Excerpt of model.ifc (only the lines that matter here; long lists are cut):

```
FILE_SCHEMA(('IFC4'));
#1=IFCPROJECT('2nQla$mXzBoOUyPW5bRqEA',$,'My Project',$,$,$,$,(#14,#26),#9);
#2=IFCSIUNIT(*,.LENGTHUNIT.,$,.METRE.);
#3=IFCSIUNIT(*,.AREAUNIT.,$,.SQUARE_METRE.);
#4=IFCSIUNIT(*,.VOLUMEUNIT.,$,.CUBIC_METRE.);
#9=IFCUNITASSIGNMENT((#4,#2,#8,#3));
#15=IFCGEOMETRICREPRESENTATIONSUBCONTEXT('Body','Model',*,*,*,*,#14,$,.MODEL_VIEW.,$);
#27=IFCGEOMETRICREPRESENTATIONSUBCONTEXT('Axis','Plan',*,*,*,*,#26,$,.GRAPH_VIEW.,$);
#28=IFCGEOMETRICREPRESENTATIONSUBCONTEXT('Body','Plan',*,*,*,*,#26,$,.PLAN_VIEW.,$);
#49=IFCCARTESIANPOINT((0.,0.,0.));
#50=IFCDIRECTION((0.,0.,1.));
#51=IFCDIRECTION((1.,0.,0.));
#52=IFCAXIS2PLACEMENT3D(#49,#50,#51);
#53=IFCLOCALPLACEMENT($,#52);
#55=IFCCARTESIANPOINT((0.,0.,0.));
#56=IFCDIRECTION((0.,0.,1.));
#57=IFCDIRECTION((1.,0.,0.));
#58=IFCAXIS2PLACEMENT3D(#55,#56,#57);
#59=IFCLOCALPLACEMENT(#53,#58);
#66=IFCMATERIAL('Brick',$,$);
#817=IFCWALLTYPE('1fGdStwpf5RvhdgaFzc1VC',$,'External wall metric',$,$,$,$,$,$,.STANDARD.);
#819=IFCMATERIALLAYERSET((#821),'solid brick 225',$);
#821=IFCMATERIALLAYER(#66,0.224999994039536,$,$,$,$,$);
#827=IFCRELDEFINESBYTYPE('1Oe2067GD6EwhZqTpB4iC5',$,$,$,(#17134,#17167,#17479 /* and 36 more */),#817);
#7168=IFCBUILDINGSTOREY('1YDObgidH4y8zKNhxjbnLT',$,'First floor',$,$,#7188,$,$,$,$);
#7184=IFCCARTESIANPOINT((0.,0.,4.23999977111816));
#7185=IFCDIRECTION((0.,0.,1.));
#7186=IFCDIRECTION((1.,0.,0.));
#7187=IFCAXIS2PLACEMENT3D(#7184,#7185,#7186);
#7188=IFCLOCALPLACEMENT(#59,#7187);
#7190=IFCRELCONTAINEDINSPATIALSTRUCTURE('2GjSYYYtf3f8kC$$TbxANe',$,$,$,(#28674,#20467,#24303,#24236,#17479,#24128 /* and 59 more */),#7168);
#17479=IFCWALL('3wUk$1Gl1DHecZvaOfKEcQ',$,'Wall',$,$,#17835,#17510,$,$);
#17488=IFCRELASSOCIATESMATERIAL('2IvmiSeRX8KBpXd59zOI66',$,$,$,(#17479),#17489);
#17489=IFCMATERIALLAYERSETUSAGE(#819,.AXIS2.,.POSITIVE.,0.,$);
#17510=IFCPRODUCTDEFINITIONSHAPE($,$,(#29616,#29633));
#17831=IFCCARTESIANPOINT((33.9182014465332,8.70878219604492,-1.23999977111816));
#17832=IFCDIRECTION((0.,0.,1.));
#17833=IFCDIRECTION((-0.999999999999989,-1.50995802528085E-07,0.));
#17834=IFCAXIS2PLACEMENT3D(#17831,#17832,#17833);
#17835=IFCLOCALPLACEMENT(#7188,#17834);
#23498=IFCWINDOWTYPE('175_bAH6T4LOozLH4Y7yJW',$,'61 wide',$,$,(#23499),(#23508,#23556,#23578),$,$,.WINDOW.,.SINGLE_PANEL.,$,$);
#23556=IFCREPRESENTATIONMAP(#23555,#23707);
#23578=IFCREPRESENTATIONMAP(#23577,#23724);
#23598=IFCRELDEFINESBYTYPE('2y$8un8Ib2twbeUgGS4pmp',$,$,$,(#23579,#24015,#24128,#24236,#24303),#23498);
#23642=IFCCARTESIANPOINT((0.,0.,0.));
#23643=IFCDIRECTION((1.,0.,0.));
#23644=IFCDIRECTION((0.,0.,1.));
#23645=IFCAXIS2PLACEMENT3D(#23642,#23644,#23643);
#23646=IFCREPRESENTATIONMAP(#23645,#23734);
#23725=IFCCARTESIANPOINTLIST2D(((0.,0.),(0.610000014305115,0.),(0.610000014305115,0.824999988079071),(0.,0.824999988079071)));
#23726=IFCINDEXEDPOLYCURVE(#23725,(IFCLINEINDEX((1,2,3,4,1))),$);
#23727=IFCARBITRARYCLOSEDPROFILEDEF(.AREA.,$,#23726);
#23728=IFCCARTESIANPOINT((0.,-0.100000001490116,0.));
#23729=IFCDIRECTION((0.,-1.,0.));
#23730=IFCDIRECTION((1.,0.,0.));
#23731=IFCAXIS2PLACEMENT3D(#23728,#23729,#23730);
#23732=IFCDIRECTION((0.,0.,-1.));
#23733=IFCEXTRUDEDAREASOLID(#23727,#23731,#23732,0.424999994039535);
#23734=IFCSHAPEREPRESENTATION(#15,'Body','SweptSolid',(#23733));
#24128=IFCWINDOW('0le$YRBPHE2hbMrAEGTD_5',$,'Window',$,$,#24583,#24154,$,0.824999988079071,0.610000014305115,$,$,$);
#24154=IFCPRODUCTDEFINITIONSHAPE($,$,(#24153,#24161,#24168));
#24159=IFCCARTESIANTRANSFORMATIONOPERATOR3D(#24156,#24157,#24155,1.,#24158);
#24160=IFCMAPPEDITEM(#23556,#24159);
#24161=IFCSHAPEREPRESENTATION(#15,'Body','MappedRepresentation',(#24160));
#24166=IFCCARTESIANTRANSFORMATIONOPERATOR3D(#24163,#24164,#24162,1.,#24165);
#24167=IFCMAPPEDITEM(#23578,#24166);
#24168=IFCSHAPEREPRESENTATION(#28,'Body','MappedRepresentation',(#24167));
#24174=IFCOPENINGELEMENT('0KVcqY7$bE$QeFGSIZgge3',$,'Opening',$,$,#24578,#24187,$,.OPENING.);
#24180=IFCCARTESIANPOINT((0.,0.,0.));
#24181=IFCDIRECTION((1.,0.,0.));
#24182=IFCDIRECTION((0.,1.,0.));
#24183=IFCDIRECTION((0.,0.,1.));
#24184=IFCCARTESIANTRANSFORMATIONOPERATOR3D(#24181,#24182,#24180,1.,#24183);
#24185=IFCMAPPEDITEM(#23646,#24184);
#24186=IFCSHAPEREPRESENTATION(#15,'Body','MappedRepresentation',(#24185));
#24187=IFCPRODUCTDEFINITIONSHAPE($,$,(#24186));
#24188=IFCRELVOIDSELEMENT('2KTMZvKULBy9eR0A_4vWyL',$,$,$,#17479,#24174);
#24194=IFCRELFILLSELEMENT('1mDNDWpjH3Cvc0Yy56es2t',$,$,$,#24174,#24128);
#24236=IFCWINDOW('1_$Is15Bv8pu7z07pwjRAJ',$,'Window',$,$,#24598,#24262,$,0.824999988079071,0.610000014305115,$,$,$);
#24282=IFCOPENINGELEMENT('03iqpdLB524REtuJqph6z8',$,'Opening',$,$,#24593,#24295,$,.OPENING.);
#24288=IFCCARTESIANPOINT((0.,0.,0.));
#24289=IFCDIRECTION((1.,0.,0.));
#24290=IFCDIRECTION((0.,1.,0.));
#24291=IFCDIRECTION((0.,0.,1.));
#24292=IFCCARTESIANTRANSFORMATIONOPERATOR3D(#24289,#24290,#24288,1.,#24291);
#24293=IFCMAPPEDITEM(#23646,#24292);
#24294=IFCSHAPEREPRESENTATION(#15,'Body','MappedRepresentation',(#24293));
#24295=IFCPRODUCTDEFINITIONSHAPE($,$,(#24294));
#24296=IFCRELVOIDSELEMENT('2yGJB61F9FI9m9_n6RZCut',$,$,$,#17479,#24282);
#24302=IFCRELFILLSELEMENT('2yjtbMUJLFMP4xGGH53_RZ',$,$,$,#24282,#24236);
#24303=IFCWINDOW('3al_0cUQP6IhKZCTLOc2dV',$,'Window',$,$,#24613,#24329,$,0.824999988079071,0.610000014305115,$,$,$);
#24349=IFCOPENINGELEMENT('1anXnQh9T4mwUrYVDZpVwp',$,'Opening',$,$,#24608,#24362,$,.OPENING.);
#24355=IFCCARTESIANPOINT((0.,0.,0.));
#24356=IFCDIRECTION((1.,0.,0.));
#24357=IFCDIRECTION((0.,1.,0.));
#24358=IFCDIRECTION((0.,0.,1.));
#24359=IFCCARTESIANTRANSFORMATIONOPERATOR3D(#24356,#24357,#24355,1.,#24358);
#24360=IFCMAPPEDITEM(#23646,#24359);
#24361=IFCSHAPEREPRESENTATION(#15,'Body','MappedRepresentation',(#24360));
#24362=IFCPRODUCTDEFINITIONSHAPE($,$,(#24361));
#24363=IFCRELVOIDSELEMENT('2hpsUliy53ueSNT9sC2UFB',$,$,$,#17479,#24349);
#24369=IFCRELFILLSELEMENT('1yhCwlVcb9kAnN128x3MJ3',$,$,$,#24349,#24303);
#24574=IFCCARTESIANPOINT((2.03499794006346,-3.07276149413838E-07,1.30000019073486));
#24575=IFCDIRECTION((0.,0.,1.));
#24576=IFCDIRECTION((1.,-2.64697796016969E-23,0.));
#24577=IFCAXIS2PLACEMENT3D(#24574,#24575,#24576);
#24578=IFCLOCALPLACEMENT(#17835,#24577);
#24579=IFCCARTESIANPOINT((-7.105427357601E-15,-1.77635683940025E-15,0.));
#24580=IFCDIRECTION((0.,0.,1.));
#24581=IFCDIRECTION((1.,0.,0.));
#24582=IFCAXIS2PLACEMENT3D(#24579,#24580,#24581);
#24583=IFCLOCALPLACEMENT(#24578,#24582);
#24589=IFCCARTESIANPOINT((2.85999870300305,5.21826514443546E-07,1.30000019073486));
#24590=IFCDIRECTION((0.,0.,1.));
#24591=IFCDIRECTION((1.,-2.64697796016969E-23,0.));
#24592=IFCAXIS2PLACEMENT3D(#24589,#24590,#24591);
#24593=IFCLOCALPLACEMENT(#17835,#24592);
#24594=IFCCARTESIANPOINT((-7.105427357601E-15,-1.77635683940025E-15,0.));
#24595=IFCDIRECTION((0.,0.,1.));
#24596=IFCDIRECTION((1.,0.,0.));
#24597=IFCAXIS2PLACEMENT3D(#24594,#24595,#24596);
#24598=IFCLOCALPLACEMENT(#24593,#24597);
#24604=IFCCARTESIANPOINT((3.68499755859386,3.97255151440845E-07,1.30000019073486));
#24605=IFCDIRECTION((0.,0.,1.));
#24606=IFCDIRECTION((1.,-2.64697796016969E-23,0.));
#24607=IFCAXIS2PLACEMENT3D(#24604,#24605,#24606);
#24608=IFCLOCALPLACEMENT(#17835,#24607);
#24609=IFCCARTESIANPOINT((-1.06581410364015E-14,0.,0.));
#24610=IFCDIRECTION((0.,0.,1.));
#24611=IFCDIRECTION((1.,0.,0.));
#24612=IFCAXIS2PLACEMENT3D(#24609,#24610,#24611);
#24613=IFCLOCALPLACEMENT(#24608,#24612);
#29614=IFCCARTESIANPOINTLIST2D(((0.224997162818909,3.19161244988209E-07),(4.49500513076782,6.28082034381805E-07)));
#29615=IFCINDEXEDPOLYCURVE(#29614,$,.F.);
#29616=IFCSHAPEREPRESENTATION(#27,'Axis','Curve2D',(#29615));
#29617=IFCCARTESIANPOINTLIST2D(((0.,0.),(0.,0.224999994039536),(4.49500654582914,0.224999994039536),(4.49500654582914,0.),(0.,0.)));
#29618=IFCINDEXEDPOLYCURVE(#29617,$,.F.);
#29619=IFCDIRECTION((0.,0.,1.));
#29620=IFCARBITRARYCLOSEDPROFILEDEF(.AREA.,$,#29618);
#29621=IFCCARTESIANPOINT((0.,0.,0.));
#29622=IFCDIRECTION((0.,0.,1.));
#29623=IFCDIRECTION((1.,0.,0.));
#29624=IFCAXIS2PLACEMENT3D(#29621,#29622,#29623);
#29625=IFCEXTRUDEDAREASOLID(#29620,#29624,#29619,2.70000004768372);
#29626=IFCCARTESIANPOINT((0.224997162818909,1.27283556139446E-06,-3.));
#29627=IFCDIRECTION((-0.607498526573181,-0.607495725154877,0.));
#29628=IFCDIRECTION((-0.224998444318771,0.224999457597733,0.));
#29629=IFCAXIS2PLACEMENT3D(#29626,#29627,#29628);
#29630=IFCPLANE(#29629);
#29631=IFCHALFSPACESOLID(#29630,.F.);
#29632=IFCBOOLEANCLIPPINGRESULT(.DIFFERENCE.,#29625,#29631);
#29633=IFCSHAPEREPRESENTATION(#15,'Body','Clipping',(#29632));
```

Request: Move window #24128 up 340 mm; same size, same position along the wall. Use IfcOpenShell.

```python
import numpy as np
import ifcopenshell
import ifcopenshell.api.geometry
import ifcopenshell.util.placement
import ifcopenshell.util.unit

model = ifcopenshell.open("model.ifc")
unit_scale = ifcopenshell.util.unit.calculate_unit_scale(model)

window = model.by_guid("0le$YRBPHE2hbMrAEGTD_5")
opening = window.FillsVoids[0].RelatingOpeningElement
dz = 0.34 / unit_scale

shift = np.array([0.0, 0.0, dz])
# The window is placed relative to its opening, so it follows when the opening moves.
matrix = ifcopenshell.util.placement.get_local_placement(opening.ObjectPlacement)
matrix[:3, 3] += shift
ifcopenshell.api.geometry.edit_object_placement(
    model, product=opening, matrix=matrix, is_si=False, should_transform_children=True
)

print(f"moved by {dz * unit_scale:+.3f} m")

model.write("model_edited.ifc")
```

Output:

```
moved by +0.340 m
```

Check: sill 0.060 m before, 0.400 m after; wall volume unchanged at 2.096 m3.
